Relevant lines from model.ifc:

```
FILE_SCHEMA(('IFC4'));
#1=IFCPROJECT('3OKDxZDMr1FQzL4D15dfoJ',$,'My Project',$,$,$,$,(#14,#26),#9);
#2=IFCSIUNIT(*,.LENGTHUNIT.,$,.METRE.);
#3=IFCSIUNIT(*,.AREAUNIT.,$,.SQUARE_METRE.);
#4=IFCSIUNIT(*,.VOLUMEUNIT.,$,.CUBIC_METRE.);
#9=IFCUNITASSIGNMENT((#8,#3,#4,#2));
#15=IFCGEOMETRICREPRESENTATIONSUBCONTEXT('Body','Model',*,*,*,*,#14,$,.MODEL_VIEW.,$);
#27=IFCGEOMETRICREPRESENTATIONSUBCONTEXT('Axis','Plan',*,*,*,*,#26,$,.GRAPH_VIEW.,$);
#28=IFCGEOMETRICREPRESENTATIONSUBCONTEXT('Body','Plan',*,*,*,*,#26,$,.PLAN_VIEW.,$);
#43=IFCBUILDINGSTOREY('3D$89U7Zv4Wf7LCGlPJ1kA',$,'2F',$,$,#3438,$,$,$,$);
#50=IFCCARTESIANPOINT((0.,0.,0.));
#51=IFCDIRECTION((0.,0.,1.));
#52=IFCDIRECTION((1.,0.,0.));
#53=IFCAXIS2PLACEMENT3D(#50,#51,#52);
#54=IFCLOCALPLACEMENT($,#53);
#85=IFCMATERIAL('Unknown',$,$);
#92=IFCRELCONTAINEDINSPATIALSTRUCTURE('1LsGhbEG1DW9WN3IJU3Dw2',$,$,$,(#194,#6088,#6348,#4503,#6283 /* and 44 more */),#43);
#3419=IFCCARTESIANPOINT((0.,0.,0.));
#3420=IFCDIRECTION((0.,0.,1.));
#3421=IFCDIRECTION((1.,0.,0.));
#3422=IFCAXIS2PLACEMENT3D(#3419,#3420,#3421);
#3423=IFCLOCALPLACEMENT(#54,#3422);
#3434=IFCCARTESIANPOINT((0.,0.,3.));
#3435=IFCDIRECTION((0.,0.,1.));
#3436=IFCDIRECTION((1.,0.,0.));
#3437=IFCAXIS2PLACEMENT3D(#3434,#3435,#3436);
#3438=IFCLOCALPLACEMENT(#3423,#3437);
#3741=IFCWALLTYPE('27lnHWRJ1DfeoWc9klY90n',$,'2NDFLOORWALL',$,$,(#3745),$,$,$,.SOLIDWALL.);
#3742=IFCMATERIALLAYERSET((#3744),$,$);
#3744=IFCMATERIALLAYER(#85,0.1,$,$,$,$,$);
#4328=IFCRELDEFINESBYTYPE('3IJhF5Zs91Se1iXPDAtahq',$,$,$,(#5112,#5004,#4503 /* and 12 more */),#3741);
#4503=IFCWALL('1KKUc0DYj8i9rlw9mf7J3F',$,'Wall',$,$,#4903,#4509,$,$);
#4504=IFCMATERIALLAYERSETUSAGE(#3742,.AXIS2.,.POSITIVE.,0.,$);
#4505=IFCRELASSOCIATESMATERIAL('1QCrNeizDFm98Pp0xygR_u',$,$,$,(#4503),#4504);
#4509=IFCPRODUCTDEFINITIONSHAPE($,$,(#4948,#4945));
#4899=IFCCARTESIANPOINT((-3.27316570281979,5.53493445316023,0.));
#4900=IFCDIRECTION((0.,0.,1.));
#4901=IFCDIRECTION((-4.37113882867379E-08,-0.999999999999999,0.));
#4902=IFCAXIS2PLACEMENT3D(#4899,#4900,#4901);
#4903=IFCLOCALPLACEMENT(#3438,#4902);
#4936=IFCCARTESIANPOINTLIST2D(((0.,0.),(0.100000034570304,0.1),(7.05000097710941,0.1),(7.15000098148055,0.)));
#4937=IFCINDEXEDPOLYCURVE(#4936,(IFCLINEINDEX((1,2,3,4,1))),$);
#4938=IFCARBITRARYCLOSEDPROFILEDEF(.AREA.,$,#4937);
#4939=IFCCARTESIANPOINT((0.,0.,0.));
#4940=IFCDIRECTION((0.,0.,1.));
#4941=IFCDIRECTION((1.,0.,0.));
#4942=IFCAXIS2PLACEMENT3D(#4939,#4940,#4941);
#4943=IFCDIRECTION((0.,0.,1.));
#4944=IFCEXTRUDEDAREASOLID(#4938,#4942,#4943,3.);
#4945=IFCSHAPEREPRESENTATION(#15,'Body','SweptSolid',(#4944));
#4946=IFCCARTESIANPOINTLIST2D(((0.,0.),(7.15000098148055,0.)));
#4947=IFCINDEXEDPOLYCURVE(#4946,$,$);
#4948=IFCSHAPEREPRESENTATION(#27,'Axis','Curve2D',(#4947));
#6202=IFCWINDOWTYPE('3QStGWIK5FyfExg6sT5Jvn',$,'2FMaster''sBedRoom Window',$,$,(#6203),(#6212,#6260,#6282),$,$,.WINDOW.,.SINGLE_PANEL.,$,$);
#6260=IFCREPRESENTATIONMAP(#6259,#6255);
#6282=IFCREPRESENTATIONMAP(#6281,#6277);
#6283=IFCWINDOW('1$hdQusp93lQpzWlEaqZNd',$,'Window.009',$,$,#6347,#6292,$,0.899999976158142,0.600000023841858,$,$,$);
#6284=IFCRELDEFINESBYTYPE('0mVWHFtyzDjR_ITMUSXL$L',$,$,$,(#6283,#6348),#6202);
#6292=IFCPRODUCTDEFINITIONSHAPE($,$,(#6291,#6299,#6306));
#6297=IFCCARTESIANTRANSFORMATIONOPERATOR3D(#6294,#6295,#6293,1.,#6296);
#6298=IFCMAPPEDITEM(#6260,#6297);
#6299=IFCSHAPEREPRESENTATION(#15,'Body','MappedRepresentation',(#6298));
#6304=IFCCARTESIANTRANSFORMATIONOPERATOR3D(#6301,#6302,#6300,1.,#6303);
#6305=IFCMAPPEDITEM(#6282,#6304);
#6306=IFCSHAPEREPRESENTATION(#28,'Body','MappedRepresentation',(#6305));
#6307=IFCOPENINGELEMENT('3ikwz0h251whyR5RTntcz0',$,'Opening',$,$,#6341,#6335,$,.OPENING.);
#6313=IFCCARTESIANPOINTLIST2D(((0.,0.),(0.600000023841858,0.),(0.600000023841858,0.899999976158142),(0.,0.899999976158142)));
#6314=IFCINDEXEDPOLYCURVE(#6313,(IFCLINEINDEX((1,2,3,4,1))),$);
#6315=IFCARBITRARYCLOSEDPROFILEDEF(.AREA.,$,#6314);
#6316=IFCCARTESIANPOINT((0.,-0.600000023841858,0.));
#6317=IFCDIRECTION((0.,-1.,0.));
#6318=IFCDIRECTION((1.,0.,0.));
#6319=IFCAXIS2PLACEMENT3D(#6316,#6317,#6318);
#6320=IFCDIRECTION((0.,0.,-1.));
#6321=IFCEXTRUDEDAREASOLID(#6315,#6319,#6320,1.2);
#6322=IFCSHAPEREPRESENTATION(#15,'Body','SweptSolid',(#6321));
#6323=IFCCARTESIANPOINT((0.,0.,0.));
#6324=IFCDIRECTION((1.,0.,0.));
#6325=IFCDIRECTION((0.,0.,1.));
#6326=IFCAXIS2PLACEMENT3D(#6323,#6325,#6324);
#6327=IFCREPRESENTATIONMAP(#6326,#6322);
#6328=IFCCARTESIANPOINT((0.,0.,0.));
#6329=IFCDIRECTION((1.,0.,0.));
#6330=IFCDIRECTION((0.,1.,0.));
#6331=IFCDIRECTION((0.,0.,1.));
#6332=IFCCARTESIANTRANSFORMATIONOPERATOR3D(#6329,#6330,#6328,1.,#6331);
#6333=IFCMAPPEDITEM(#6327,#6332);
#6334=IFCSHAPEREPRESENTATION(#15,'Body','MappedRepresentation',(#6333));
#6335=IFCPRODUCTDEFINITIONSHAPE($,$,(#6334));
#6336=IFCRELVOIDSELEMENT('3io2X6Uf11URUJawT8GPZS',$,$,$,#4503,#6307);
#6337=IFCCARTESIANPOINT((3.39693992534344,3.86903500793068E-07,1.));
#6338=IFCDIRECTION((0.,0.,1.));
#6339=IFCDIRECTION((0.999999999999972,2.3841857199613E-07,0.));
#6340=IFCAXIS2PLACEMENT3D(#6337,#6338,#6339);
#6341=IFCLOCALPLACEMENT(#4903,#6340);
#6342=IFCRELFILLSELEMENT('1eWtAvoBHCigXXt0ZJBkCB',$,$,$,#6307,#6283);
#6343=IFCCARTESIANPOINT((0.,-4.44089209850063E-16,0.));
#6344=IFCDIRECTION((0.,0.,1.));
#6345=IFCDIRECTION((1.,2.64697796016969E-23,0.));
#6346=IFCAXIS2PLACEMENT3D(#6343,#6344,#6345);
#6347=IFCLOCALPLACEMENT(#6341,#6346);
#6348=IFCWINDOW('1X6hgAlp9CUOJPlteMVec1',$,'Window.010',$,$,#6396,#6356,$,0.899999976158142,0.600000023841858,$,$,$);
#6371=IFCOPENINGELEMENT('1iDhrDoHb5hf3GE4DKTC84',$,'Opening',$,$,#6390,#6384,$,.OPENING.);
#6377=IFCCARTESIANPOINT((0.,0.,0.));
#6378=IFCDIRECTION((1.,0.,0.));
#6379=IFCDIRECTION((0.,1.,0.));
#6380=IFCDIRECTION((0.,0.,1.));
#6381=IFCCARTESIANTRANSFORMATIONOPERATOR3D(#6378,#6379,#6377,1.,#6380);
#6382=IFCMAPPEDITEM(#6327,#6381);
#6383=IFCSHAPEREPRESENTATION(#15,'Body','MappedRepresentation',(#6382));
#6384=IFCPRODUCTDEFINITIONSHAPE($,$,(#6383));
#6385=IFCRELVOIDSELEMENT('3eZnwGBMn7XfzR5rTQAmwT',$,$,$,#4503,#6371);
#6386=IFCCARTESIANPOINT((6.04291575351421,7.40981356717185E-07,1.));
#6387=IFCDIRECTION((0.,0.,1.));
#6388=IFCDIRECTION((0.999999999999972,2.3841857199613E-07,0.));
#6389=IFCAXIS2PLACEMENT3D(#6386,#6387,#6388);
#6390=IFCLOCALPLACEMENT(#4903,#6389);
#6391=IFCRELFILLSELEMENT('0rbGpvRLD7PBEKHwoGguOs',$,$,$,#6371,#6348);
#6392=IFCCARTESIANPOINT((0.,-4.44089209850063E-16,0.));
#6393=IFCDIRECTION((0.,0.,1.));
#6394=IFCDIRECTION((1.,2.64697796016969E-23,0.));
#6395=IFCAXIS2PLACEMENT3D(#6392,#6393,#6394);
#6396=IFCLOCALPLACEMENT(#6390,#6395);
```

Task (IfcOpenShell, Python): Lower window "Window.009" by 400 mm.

```python
import numpy as np
import ifcopenshell
import ifcopenshell.api.geometry
import ifcopenshell.util.placement
import ifcopenshell.util.unit

model = ifcopenshell.open("model.ifc")
unit_scale = ifcopenshell.util.unit.calculate_unit_scale(model)

window = model.by_guid("1$hdQusp93lQpzWlEaqZNd")
opening = window.FillsVoids[0].RelatingOpeningElement
dz = -0.4 / unit_scale

shift = np.array([0.0, 0.0, dz])
# The window is placed relative to its opening, so it follows when the opening moves.
matrix = ifcopenshell.util.placement.get_local_placement(opening.ObjectPlacement)
matrix[:3, 3] += shift
ifcopenshell.api.geometry.edit_object_placement(
    model, product=opening, matrix=matrix, is_si=False, should_transform_children=True
)

print(f"moved by {dz * unit_scale:+.3f} m")

model.write("model_rev.ifc")
```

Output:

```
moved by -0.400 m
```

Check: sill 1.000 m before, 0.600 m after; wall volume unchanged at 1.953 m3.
